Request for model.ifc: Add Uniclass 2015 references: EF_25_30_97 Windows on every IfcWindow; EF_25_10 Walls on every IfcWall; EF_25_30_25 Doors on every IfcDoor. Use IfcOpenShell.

First a look at what the model holds.

```python
import ifcopenshell

model = ifcopenshell.open("model.ifc")
print(model.schema)
print("classifications:", [c.Name for c in model.by_type("IfcClassification")])
for ifc_class in ("IfcDoor", "IfcRoof", "IfcStair", "IfcWall", "IfcWindow"):
    print(ifc_class, len(model.by_type(ifc_class)))
```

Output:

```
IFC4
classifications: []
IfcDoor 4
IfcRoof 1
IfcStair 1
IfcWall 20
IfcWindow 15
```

```python
import ifcopenshell
import ifcopenshell.api.classification

model = ifcopenshell.open("model.ifc")

system = ifcopenshell.api.classification.add_classification(model, classification="Uniclass 2015")

codes = {
    "IfcWindow": ("EF_25_30_97", "Windows"),
    "IfcWall": ("EF_25_10", "Walls"),
    "IfcDoor": ("EF_25_30_25", "Doors"),
}
for ifc_class, (code, name) in codes.items():
    products = model.by_type(ifc_class)
    ifcopenshell.api.classification.add_reference(
        model, products=products, classification=system, identification=code, name=name
    )
    print(code, len(products))

model.write("model_updated.ifc")
```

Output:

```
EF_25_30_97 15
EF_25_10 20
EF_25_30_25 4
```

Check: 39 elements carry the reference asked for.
